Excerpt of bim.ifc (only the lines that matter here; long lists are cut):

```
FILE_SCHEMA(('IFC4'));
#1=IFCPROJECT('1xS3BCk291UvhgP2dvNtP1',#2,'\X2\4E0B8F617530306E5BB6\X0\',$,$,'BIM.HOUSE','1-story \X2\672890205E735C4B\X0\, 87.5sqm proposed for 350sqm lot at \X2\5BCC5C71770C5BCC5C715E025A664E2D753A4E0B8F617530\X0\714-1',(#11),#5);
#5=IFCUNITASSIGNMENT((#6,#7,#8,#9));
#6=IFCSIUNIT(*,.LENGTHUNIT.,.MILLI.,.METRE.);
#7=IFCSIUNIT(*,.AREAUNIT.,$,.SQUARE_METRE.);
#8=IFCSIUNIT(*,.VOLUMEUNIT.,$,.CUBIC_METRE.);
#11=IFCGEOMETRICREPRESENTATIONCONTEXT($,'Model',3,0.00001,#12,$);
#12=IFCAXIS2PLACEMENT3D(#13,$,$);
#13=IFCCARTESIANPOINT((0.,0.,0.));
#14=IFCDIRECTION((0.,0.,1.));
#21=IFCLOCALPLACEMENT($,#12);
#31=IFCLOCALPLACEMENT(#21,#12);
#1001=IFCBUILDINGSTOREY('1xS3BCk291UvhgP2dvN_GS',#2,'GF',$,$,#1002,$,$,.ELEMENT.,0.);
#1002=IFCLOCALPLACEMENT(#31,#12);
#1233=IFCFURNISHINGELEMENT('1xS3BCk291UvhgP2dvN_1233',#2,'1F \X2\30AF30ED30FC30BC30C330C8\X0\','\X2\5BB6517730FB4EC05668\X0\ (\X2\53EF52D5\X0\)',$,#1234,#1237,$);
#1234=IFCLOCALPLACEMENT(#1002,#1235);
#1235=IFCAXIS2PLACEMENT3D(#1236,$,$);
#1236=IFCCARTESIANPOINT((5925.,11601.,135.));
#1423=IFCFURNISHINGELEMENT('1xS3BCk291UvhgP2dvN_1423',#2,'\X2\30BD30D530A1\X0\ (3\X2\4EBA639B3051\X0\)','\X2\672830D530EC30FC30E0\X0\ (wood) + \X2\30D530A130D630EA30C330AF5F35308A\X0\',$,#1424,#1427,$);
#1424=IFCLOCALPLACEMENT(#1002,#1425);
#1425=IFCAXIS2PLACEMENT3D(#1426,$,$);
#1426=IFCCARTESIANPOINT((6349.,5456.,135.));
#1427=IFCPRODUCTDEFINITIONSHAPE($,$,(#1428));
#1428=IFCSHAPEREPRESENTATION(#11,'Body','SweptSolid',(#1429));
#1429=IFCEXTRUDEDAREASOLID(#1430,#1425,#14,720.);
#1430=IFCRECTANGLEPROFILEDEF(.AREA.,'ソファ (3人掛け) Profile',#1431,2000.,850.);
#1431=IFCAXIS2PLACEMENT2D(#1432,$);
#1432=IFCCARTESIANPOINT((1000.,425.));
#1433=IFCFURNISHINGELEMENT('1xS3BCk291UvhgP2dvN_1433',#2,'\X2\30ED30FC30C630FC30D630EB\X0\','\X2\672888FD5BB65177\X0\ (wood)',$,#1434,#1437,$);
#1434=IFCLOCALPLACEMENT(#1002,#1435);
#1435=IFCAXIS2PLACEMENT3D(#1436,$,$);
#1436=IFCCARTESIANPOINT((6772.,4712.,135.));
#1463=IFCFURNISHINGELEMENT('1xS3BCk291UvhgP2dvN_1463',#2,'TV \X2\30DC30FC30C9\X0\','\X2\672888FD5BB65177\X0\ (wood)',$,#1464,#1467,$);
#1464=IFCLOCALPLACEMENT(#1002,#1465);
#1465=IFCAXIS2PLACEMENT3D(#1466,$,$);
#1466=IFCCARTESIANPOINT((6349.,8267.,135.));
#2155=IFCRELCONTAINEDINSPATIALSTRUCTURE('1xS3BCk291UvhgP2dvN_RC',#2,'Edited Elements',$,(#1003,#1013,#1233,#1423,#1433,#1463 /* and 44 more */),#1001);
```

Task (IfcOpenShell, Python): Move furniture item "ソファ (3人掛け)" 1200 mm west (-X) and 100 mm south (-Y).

```python
import ifcopenshell
import ifcopenshell.api.geometry
import ifcopenshell.util.placement
import ifcopenshell.util.unit

model = ifcopenshell.open("bim.ifc")
unit_scale = ifcopenshell.util.unit.calculate_unit_scale(model)

item = model.by_guid("1xS3BCk291UvhgP2dvN_1423")
matrix = ifcopenshell.util.placement.get_local_placement(item.ObjectPlacement)
matrix[0, 3] -= 1.2 / unit_scale
matrix[1, 3] -= 0.1 / unit_scale
ifcopenshell.api.geometry.edit_object_placement(model, product=item, matrix=matrix, is_si=False)

print(ifcopenshell.util.placement.get_local_placement(item.ObjectPlacement).round(3) + 0.0)

model.write("bim_edited.ifc")
```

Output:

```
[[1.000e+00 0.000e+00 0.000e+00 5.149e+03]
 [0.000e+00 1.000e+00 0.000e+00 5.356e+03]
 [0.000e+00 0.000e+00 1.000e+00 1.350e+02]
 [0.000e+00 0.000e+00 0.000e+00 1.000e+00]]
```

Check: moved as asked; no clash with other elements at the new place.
